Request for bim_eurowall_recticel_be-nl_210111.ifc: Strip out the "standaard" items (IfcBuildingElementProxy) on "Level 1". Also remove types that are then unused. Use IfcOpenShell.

First a look at what the model holds.

```python
import ifcopenshell
import ifcopenshell.util.element

model = ifcopenshell.open("bim_eurowall_recticel_be-nl_210111.ifc")
print(model.schema)
storey = next(s for s in model.by_type("IfcBuildingStorey") if s.Name == "Level 1")
proxies = [e for e in ifcopenshell.util.element.get_decomposition(storey) if e.is_a("IfcBuildingElementProxy")]
seen = {}
for e in proxies:
    element_type = ifcopenshell.util.element.get_type(e)
    name = element_type.Name if element_type not in (None, e) else None
    seen[name] = seen.get(name, 0) + 1
for name, count in sorted(seen.items(), key=str):
    print(count, "x", name)
```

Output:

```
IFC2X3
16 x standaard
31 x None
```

```python
import ifcopenshell
import ifcopenshell.api.root
import ifcopenshell.util.element

model = ifcopenshell.open("bim_eurowall_recticel_be-nl_210111.ifc")

storey = next(s for s in model.by_type("IfcBuildingStorey") if s.Name == "Level 1")
proxies = [e for e in ifcopenshell.util.element.get_decomposition(storey) if e.is_a("IfcBuildingElementProxy")]
targets = [e for e in proxies if (t := ifcopenshell.util.element.get_type(e)) not in (None, e) and t.Name == "standaard"]
types = {ifcopenshell.util.element.get_type(e) for e in targets} - {None, *targets}

for e in targets:
    ifcopenshell.api.root.remove_product(model, product=e)
print(len(targets), "removed")

unused = [t for t in types if not ifcopenshell.util.element.get_types(t)]
for t in unused:
    ifcopenshell.api.root.remove_product(model, product=t)
print(len(unused), "unused types removed")

model.write("bim_eurowall_recticel_be-nl_210111_v2.ifc")
```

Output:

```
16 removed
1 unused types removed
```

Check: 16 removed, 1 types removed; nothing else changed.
